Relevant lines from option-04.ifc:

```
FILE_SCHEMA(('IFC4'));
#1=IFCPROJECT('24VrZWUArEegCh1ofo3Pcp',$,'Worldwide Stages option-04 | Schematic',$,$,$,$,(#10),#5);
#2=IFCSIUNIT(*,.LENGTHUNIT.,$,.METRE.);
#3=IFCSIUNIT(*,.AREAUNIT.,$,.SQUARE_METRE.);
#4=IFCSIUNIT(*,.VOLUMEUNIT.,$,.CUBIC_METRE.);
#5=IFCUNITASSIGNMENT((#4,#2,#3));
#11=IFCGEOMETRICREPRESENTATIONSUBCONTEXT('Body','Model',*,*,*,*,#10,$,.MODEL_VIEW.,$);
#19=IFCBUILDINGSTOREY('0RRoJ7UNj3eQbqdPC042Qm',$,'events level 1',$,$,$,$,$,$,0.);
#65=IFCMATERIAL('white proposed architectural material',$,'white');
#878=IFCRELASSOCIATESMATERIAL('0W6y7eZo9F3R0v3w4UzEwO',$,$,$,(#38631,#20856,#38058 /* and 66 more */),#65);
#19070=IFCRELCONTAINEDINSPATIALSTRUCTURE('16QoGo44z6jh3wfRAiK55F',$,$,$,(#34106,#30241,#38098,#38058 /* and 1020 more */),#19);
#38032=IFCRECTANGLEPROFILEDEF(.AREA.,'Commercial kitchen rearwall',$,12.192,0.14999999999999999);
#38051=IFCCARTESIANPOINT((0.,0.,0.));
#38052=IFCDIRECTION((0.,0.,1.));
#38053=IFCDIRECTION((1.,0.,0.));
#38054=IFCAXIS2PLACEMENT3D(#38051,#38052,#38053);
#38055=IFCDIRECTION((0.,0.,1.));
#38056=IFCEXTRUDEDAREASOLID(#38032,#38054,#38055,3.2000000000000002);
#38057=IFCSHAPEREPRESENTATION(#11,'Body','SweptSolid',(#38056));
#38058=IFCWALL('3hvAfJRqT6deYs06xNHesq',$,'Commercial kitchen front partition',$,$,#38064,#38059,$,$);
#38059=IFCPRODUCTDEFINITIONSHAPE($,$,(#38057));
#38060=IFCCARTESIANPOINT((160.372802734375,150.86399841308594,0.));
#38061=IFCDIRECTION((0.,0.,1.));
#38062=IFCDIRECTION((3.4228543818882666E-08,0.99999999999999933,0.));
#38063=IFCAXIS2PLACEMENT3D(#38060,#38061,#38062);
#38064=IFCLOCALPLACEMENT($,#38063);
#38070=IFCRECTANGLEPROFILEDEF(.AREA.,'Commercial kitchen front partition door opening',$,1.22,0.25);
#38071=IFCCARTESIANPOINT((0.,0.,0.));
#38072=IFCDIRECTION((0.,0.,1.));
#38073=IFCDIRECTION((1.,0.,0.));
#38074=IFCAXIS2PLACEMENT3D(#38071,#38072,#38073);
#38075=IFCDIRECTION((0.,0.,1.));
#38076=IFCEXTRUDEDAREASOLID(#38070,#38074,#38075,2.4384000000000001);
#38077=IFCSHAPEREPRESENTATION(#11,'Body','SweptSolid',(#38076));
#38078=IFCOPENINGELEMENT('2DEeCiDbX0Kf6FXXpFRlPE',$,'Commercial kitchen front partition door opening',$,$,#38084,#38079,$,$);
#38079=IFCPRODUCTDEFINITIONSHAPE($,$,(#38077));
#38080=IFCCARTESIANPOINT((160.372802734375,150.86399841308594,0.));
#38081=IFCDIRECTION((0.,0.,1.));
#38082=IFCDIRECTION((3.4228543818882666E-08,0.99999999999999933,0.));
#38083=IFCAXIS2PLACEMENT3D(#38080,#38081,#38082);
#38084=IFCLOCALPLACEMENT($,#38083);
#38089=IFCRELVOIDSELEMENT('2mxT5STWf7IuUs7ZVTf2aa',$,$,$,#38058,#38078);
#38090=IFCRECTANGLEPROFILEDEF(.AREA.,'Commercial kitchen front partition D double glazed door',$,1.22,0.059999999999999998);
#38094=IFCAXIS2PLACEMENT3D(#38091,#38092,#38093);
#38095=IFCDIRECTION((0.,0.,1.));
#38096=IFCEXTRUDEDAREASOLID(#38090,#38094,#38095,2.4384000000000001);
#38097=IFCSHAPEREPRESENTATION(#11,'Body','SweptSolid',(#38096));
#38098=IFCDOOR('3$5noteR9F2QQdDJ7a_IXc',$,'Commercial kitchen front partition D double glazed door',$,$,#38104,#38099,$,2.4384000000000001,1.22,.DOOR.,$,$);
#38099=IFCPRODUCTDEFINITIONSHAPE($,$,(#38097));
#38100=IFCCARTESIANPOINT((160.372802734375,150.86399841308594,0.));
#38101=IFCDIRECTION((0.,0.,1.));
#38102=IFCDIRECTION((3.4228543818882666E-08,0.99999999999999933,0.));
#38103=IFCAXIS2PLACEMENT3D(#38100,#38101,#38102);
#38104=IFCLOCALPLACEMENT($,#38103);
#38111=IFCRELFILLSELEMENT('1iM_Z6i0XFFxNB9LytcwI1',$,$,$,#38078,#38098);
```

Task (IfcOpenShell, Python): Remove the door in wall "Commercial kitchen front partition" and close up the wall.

```python
import ifcopenshell
import ifcopenshell.api.feature
import ifcopenshell.api.root
import ifcopenshell.geom
import ifcopenshell.util.shape

model = ifcopenshell.open("option-04.ifc")
settings = ifcopenshell.geom.settings()


def volume(element):
    """Net volume in cubic metres, openings subtracted."""
    shape = ifcopenshell.geom.create_shape(settings, element)
    return ifcopenshell.util.shape.get_volume(shape.geometry)


door = model.by_guid("3$5noteR9F2QQdDJ7a_IXc")
opening = door.FillsVoids[0].RelatingOpeningElement
wall = opening.VoidsElements[0].RelatingBuildingElement
before = volume(wall)

ifcopenshell.api.root.remove_product(model, product=door)
ifcopenshell.api.feature.remove_feature(model, feature=opening)

after = volume(wall)

print(f"wall volume {before:.3f} -> {after:.3f} m3")

model.write("option-04_v2.ifc")
```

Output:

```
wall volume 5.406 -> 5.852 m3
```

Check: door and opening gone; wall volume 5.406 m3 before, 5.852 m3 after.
